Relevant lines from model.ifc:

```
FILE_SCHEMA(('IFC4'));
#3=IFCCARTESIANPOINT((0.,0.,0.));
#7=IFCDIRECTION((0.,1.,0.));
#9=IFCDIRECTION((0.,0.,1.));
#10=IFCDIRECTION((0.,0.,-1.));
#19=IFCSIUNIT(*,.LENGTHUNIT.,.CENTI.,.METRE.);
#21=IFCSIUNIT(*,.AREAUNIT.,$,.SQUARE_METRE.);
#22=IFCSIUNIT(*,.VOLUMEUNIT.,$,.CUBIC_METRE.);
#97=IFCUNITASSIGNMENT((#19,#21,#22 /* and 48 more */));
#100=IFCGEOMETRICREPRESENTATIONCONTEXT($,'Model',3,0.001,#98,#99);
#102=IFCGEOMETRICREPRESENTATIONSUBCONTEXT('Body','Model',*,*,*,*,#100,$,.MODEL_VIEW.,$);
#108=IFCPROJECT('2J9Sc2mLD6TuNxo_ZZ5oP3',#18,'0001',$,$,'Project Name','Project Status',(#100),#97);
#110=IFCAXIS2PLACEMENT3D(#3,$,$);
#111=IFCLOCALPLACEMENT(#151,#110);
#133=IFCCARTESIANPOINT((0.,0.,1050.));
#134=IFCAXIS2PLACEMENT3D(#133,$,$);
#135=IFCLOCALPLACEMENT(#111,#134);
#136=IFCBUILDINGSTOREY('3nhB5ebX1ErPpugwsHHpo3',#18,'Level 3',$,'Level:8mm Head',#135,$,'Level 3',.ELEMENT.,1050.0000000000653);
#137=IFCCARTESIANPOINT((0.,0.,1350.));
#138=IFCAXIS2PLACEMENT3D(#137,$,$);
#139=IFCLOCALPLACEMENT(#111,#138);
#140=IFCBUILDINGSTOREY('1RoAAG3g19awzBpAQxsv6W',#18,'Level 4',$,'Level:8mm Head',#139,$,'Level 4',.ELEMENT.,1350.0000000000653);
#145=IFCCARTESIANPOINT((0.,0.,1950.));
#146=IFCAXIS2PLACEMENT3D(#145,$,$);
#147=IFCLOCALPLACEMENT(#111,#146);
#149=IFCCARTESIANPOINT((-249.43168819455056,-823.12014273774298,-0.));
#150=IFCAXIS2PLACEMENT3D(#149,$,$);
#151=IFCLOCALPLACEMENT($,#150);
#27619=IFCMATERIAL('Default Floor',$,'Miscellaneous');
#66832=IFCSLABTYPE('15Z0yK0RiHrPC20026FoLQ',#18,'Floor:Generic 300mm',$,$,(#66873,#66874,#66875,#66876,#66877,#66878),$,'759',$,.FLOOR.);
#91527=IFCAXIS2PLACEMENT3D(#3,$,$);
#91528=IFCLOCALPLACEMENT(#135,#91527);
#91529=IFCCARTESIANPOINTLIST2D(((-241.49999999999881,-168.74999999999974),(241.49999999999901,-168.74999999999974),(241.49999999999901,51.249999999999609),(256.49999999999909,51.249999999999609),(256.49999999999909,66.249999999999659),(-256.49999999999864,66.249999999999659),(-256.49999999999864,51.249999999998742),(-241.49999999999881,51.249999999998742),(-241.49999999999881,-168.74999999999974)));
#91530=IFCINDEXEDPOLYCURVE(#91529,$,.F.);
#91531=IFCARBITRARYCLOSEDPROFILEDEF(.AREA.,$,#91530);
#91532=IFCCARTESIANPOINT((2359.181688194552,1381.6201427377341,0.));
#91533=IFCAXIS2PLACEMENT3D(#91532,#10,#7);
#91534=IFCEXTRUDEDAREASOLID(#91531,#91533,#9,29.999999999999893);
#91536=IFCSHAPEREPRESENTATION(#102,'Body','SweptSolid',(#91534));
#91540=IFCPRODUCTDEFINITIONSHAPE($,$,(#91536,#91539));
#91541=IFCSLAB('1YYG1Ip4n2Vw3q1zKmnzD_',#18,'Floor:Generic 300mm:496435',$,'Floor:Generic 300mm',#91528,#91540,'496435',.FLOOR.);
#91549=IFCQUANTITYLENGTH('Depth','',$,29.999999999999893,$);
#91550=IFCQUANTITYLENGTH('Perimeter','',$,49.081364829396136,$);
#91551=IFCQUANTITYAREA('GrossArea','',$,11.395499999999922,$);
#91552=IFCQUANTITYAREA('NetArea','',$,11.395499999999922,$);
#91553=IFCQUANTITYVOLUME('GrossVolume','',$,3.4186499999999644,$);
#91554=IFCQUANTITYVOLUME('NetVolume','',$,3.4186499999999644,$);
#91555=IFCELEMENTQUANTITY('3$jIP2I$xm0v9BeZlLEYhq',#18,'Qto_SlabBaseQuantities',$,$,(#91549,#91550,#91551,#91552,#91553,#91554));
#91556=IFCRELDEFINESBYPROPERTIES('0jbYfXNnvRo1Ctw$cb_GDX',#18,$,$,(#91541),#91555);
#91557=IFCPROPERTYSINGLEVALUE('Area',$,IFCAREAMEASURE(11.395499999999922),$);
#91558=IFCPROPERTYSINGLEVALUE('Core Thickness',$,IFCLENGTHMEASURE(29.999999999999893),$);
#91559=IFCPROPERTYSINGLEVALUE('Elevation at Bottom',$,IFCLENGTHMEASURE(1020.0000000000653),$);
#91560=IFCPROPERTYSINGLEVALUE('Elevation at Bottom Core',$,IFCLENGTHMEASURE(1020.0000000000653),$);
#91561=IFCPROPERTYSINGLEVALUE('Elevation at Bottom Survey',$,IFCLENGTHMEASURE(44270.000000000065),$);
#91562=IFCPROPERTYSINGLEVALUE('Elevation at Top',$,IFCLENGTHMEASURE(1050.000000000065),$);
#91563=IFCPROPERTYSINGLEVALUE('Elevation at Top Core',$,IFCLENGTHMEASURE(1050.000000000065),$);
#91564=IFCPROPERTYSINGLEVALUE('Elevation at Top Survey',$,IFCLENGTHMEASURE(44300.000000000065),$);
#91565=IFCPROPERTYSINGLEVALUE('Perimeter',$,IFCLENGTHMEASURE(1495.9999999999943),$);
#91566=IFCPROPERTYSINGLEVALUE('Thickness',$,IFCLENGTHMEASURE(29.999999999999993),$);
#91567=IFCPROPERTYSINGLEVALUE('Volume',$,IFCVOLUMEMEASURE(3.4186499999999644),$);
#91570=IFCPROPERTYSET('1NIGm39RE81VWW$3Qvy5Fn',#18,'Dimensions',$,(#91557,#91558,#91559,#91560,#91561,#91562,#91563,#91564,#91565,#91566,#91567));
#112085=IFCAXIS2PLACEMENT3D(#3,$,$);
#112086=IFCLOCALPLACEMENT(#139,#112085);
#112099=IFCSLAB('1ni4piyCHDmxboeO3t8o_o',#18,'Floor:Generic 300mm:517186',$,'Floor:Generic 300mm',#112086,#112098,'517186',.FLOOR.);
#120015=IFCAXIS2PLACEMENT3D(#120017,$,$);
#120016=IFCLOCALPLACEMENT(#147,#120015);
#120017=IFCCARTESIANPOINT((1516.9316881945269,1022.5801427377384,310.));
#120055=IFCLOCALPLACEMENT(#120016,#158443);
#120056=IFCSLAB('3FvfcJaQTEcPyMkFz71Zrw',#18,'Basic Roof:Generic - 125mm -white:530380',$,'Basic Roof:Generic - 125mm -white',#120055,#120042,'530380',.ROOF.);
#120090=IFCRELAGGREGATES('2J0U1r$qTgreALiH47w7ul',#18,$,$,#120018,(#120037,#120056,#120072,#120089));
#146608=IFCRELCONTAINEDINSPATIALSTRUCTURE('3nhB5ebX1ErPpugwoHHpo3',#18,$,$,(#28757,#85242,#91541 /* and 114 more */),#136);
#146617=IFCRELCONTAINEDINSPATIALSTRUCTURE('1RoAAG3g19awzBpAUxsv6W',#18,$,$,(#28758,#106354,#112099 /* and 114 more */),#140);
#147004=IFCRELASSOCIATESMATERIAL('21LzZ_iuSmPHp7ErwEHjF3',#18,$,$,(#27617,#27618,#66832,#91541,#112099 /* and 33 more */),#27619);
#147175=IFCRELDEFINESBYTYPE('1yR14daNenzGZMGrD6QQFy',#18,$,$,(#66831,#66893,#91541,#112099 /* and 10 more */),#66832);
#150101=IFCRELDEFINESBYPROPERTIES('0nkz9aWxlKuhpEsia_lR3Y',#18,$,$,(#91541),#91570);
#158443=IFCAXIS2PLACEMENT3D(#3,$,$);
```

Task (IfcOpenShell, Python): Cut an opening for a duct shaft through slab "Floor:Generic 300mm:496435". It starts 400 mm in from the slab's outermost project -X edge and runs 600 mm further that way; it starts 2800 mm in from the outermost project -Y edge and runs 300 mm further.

```python
import numpy as np
import ifcopenshell
import ifcopenshell.api.feature
import ifcopenshell.api.geometry
import ifcopenshell.api.pset
import ifcopenshell.api.root
import ifcopenshell.geom
import ifcopenshell.util.element
import ifcopenshell.util.placement
import ifcopenshell.util.representation
import ifcopenshell.util.shape
import ifcopenshell.util.unit

model = ifcopenshell.open("model.ifc")
unit_scale = ifcopenshell.util.unit.calculate_unit_scale(model)
area_scale = ifcopenshell.util.unit.calculate_unit_scale(model, "AREAUNIT")
volume_scale = ifcopenshell.util.unit.calculate_unit_scale(model, "VOLUMEUNIT")
settings = ifcopenshell.geom.settings()


def volume(element):
    """Net volume in cubic metres, openings subtracted."""
    shape = ifcopenshell.geom.create_shape(settings, element)
    return ifcopenshell.util.shape.get_volume(shape.geometry)


slab = model.by_guid("1YYG1Ip4n2Vw3q1zKmnzD_")
before = volume(slab)

# Extent in the slab's own axes, in metres. The edges named are its -X and -Y sides.
slab_shape = ifcopenshell.geom.create_shape(settings, slab)
vertices = ifcopenshell.util.shape.get_vertices(slab_shape.geometry)
x_min, y_min, bottom = vertices.min(axis=0)
top = vertices[:, 2].max()

opening = ifcopenshell.api.root.create_entity(model, ifc_class="IfcOpeningElement", name="Duct shaft opening", predefined_type="OPENING")
context = ifcopenshell.util.representation.get_context(model, "Model", "Body", "MODEL_VIEW")
width, depth = 0.6, 0.3
outline = [(0.0, 0.0), (width, 0.0), (width, depth), (0.0, depth), (0.0, 0.0)]
# Overshoot both faces by 50 mm so the cut is clean.
shape = ifcopenshell.api.geometry.add_slab_representation(
    model, context=context, depth=top - bottom + 0.1, polyline=outline
)
ifcopenshell.api.geometry.assign_representation(model, product=opening, representation=shape)

matrix = ifcopenshell.util.placement.get_local_placement(slab.ObjectPlacement)
matrix[:, 3] = matrix @ np.append(np.array([x_min + 0.4, y_min + 2.8, bottom - 0.05]) / unit_scale, 1.0)
ifcopenshell.api.geometry.edit_object_placement(model, product=opening, matrix=matrix, is_si=False)
ifcopenshell.api.feature.add_feature(model, feature=opening, element=slab)

after = volume(slab)

# Update the slab's stored quantities.
qto = model.by_id(ifcopenshell.util.element.get_pset(slab, "Qto_SlabBaseQuantities", should_inherit=False)["id"])
ifcopenshell.api.pset.edit_qto(model, qto=qto, properties={
    "NetArea": after / (top - bottom) / area_scale,
    "NetVolume": after / volume_scale,
})
pset = model.by_id(ifcopenshell.util.element.get_pset(slab, "Dimensions", should_inherit=False)["id"])
ifcopenshell.api.pset.edit_pset(model, pset=pset, properties={
    "Area": model.create_entity("IfcAreaMeasure", after / (top - bottom) / area_scale),
    "Volume": model.create_entity("IfcVolumeMeasure", after / volume_scale),
})

print(f"slab volume {before:.3f} -> {after:.3f} m3")

model.write("model_rev.ifc")
```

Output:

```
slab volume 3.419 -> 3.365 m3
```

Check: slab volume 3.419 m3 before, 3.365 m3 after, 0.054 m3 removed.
